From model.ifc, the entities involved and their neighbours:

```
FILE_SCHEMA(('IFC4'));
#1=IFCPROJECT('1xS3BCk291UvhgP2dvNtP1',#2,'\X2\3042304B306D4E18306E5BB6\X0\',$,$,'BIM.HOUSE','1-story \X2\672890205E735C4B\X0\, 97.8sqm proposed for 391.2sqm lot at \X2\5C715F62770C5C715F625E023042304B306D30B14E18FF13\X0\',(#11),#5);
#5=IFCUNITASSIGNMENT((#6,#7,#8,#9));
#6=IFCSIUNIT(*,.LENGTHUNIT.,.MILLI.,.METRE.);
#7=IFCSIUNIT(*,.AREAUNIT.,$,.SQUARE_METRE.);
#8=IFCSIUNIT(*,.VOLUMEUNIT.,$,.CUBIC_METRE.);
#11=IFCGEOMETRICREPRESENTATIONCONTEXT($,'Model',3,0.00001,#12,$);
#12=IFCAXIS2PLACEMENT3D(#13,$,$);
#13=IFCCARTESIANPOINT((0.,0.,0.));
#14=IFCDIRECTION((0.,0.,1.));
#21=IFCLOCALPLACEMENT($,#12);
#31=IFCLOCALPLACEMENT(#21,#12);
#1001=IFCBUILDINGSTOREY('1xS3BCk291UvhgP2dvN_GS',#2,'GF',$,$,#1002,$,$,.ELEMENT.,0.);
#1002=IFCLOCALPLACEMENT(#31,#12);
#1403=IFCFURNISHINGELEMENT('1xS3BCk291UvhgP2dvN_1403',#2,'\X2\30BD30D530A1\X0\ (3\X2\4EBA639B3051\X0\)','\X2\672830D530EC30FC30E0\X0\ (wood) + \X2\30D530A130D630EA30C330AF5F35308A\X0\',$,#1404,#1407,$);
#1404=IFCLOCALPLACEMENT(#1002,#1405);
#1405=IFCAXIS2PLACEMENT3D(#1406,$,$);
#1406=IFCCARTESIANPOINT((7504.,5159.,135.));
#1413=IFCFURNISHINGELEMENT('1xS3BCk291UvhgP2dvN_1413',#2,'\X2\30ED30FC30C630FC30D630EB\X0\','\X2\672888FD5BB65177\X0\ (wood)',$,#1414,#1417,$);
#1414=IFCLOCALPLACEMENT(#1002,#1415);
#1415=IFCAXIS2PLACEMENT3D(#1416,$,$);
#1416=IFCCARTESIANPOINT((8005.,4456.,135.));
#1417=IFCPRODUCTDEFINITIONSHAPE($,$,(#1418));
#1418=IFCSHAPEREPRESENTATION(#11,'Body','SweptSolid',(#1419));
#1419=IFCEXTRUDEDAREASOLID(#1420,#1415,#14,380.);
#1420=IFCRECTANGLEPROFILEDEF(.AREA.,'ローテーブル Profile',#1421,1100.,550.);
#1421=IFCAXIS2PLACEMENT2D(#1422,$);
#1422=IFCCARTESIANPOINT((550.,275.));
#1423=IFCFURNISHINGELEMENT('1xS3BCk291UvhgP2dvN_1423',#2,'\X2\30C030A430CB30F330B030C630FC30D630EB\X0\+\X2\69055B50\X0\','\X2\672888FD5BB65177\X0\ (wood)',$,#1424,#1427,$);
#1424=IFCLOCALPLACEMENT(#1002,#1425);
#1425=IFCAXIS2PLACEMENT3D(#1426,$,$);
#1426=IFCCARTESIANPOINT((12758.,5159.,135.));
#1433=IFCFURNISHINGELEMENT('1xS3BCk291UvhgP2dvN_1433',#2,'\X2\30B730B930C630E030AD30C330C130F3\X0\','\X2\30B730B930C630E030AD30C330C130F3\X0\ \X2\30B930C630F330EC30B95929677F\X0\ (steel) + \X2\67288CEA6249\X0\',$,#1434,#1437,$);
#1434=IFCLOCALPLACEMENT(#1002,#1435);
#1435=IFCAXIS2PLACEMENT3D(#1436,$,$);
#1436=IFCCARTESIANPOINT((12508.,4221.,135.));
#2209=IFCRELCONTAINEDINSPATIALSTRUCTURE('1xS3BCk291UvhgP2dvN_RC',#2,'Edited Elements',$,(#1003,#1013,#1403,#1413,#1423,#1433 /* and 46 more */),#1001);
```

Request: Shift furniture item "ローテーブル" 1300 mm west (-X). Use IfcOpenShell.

```python
import ifcopenshell
import ifcopenshell.api.geometry
import ifcopenshell.util.placement
import ifcopenshell.util.unit

model = ifcopenshell.open("model.ifc")
unit_scale = ifcopenshell.util.unit.calculate_unit_scale(model)

item = model.by_guid("1xS3BCk291UvhgP2dvN_1413")
matrix = ifcopenshell.util.placement.get_local_placement(item.ObjectPlacement)
matrix[0, 3] -= 1.3 / unit_scale
ifcopenshell.api.geometry.edit_object_placement(model, product=item, matrix=matrix, is_si=False)

print(ifcopenshell.util.placement.get_local_placement(item.ObjectPlacement).round(3) + 0.0)

model.write("model-out.ifc")
```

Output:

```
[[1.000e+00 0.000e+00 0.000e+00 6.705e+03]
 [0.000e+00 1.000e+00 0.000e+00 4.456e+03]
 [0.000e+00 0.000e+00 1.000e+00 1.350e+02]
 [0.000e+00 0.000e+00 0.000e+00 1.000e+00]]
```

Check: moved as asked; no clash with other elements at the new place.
